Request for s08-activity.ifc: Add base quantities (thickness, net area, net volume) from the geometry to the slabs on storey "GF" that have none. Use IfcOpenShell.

First a look at what the model holds.

```python
import ifcopenshell
import ifcopenshell.util.element
import ifcopenshell.util.unit

model = ifcopenshell.open("s08-activity.ifc")
print(model.schema)
for unit_type in ("LENGTHUNIT", "AREAUNIT", "VOLUMEUNIT"):
    print(unit_type, ifcopenshell.util.unit.calculate_unit_scale(model, unit_type))
storey = next(s for s in model.by_type("IfcBuildingStorey") if s.Name == "GF")
slabs = [e for e in ifcopenshell.util.element.get_decomposition(storey) if e.is_a("IfcSlab")]
for e in sorted(slabs, key=lambda e: e.id()):
    print(e.id(), e.is_a(), e.Name, list(ifcopenshell.util.element.get_psets(e, qtos_only=True)), sep=" | ")
```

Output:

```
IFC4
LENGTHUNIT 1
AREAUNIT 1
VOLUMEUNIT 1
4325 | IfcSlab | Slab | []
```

```python
import ifcopenshell
import ifcopenshell.api.pset
import ifcopenshell.geom
import ifcopenshell.util.element
import ifcopenshell.util.shape
import ifcopenshell.util.unit

model = ifcopenshell.open("s08-activity.ifc")
unit_scale = ifcopenshell.util.unit.calculate_unit_scale(model)
area_scale = ifcopenshell.util.unit.calculate_unit_scale(model, "AREAUNIT")
volume_scale = ifcopenshell.util.unit.calculate_unit_scale(model, "VOLUMEUNIT")
settings = ifcopenshell.geom.settings()

storey = next(s for s in model.by_type("IfcBuildingStorey") if s.Name == "GF")
slabs = [e for e in ifcopenshell.util.element.get_decomposition(storey) if e.is_a("IfcSlab")]

for e in sorted(slabs, key=lambda e: e.id()):
    if ifcopenshell.util.element.get_psets(e, qtos_only=True, should_inherit=False):
        continue
    # Geometry comes back in metres, in the element's own axes.
    shape = ifcopenshell.geom.create_shape(settings, e)
    values = {
        "Width": ifcopenshell.util.shape.get_z(shape.geometry) / unit_scale,
        "NetArea": ifcopenshell.util.shape.get_footprint_area(shape.geometry) / area_scale,
        "NetVolume": ifcopenshell.util.shape.get_volume(shape.geometry) / volume_scale,
    }
    qto = ifcopenshell.api.pset.add_qto(model, product=e, name="Qto_SlabBaseQuantities")
    ifcopenshell.api.pset.edit_qto(model, qto=qto, properties=values)
    print(e.id(), {k: round(v, 3) for k, v in values.items()})

model.write("s08-activity-out.ifc")
```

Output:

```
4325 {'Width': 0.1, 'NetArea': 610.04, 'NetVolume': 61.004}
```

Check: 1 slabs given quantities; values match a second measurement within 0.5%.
